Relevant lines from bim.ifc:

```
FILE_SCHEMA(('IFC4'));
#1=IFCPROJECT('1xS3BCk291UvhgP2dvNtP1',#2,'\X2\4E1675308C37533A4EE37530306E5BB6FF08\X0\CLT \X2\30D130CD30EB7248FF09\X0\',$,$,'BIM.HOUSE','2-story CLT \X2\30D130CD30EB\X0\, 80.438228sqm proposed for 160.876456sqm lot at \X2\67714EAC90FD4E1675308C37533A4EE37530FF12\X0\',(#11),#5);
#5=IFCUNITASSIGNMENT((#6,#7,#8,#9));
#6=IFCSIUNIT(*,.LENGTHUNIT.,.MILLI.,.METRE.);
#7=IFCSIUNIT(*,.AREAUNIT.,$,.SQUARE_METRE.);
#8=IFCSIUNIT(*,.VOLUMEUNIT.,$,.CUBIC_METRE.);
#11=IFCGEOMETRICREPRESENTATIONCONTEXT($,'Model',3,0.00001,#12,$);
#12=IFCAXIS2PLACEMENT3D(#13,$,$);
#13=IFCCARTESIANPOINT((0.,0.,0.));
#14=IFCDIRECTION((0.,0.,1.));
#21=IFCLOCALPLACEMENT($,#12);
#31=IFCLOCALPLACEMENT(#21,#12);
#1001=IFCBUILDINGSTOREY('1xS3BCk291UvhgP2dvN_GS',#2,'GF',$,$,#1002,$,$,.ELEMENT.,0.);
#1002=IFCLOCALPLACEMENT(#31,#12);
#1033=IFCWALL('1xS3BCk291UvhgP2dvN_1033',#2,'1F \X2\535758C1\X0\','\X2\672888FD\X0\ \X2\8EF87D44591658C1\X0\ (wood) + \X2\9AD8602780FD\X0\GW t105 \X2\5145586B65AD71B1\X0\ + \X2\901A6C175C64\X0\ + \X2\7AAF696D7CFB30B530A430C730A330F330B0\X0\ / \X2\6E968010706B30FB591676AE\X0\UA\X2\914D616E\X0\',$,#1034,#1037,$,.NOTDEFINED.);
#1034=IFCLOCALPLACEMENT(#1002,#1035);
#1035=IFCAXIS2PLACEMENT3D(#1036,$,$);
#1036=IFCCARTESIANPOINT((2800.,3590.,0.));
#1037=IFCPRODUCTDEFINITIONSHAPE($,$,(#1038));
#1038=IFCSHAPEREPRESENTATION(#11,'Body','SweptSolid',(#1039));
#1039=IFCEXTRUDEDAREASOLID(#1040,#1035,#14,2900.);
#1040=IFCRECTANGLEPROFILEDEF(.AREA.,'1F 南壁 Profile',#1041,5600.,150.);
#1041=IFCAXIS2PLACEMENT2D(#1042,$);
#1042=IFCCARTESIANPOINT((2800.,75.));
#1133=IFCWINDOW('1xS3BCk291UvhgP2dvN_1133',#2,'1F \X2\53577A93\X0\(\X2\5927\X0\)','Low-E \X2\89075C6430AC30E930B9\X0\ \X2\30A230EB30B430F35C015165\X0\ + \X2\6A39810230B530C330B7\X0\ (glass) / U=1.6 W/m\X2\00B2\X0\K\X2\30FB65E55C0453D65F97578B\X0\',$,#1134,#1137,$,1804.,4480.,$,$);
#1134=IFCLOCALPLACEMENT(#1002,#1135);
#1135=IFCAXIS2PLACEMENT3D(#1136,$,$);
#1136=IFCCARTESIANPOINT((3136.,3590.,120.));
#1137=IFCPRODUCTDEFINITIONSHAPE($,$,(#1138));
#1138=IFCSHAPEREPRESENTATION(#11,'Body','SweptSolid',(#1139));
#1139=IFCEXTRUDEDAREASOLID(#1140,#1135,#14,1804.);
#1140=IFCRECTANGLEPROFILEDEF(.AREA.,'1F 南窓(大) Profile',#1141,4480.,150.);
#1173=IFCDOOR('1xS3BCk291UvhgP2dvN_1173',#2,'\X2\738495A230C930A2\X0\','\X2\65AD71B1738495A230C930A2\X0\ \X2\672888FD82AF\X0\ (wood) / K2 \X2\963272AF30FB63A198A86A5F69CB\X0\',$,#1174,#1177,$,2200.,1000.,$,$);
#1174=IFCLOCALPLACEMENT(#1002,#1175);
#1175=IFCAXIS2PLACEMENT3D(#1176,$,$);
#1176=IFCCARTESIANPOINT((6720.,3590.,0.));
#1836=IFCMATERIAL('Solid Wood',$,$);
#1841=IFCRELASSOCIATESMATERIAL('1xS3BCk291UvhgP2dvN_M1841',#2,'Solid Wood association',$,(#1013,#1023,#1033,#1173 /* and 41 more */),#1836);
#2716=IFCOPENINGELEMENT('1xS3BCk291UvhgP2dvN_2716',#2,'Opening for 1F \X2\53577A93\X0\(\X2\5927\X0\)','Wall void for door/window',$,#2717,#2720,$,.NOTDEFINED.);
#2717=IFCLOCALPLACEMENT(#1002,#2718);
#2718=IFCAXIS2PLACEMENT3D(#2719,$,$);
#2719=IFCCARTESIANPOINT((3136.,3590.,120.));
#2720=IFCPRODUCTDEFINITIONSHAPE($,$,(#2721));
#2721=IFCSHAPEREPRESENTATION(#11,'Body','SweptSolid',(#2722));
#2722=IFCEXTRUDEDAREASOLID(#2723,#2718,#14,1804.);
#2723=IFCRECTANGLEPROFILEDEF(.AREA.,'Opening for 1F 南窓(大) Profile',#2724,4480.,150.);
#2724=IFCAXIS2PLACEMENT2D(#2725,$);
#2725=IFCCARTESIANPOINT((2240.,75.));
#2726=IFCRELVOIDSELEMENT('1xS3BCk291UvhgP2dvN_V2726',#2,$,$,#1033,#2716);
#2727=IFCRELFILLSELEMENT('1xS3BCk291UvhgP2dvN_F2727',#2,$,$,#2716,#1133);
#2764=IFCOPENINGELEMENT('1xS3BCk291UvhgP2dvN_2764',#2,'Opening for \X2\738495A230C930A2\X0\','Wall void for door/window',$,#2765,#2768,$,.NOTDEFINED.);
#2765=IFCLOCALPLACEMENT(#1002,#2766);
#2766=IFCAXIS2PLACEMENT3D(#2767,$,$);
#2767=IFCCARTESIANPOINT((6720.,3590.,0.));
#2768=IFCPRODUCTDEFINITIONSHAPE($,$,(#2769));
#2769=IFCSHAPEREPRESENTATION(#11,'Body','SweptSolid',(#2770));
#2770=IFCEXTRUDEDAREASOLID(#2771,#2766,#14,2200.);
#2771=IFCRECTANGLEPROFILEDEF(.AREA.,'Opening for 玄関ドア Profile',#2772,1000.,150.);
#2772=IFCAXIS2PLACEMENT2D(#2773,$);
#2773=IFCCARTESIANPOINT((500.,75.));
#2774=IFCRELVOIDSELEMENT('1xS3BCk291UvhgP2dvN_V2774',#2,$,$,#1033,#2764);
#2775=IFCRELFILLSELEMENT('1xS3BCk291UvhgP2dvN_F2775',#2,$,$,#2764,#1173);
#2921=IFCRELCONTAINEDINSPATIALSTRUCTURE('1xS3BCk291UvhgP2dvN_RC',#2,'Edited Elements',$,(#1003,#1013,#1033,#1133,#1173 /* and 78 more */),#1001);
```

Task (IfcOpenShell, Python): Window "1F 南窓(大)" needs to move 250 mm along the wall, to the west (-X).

```python
import ifcopenshell
import ifcopenshell.api.geometry
import ifcopenshell.util.placement
import ifcopenshell.util.unit

model = ifcopenshell.open("bim.ifc")
unit_scale = ifcopenshell.util.unit.calculate_unit_scale(model)

window = model.by_id(1133)
opening = window.FillsVoids[0].RelatingOpeningElement
wall = opening.VoidsElements[0].RelatingBuildingElement

wall_matrix = ifcopenshell.util.placement.get_local_placement(wall.ObjectPlacement)
shift = wall_matrix[:3, 0] * -0.25 / unit_scale
before = ifcopenshell.util.placement.get_local_placement(window.ObjectPlacement)[:3, 3].copy()

# The window is not placed relative to its opening, so move both.
for product in (opening, window):
    matrix = ifcopenshell.util.placement.get_local_placement(product.ObjectPlacement)
    matrix[:3, 3] += shift
    ifcopenshell.api.geometry.edit_object_placement(model, product=product, matrix=matrix, is_si=False)

after = ifcopenshell.util.placement.get_local_placement(window.ObjectPlacement)[:3, 3]
print("window moved by", (after - before).round(3) + 0.0)

model.write("bim-out.ifc")
```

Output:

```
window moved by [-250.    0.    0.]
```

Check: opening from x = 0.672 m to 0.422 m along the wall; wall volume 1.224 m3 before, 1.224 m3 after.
